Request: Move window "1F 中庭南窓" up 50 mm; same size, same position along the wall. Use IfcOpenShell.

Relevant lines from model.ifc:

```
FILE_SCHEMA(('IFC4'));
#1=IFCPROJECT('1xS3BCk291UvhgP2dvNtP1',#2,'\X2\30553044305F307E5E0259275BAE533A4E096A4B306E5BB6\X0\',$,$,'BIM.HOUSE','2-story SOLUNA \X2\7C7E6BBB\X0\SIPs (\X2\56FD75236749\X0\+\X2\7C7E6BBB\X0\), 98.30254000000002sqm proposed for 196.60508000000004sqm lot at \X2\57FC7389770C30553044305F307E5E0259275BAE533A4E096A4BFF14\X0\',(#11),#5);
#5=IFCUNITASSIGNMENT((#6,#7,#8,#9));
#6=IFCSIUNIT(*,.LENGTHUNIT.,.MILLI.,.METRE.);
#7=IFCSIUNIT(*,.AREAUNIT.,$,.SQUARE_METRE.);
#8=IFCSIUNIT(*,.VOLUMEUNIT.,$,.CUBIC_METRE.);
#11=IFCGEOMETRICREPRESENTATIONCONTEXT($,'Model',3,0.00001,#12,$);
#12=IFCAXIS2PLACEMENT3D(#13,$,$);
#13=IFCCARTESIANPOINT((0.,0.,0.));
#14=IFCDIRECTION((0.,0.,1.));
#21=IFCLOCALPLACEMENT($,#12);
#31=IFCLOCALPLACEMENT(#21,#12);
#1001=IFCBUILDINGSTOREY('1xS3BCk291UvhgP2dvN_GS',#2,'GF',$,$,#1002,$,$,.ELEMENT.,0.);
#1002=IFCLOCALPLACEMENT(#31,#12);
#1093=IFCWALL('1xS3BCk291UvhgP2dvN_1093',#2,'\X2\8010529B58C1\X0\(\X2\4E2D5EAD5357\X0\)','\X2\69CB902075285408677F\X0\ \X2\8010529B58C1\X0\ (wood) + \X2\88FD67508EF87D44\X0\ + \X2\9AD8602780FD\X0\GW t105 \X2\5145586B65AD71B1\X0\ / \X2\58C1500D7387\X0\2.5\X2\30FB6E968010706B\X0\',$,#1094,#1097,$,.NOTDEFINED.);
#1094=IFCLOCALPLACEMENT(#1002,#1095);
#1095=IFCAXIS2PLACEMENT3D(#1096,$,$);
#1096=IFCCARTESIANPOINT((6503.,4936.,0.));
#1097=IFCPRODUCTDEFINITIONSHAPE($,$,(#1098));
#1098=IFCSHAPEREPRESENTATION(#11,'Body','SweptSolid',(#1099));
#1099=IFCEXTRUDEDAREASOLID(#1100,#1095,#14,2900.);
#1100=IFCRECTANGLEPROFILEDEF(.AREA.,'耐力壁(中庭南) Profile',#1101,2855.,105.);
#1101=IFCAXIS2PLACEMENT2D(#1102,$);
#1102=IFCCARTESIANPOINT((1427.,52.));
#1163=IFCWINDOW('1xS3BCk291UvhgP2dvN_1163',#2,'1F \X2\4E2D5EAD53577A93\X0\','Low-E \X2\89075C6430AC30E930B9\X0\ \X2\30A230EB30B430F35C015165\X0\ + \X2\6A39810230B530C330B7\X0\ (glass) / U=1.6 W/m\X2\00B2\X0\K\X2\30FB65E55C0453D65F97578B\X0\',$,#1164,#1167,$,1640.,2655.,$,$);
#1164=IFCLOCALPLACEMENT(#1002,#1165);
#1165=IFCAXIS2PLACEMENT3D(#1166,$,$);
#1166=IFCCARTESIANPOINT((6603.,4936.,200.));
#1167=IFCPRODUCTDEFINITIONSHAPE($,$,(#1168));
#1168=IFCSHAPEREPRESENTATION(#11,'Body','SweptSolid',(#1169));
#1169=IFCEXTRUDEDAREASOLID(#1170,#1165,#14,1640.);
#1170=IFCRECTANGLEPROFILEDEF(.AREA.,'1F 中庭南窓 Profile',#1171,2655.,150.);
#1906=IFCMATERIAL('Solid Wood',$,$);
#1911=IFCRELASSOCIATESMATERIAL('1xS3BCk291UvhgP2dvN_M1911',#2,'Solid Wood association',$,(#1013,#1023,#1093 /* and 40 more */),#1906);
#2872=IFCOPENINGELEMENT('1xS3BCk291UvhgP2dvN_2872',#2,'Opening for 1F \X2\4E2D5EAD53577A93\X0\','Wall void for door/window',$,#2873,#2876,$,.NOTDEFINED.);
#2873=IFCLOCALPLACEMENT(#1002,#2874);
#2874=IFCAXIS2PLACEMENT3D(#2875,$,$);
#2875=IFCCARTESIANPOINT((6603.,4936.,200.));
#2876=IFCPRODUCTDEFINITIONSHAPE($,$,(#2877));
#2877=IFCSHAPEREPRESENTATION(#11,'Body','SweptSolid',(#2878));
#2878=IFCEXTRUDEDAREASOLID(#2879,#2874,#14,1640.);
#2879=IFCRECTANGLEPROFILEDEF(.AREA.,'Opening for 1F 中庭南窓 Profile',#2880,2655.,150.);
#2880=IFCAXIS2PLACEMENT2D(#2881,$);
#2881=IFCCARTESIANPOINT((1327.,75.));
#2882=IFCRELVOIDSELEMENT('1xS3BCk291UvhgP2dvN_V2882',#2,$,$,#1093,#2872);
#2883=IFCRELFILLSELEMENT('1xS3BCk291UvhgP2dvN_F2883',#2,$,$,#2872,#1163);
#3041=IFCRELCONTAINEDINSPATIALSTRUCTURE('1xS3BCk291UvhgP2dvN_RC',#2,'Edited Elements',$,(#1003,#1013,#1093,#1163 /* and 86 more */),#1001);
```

```python
import numpy as np
import ifcopenshell
import ifcopenshell.api.geometry
import ifcopenshell.util.placement
import ifcopenshell.util.unit

model = ifcopenshell.open("model.ifc")
unit_scale = ifcopenshell.util.unit.calculate_unit_scale(model)

window = model.by_guid("1xS3BCk291UvhgP2dvN_1163")
opening = window.FillsVoids[0].RelatingOpeningElement
dz = 50.0

shift = np.array([0.0, 0.0, dz])
# The window is not placed relative to its opening, so move both.
for product in (opening, window):
    matrix = ifcopenshell.util.placement.get_local_placement(product.ObjectPlacement)
    matrix[:3, 3] += shift
    ifcopenshell.api.geometry.edit_object_placement(model, product=product, matrix=matrix, is_si=False)

print(f"moved by {dz * unit_scale:+.3f} m")

model.write("model_v2.ifc")
```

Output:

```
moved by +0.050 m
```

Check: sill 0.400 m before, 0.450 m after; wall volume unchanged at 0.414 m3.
